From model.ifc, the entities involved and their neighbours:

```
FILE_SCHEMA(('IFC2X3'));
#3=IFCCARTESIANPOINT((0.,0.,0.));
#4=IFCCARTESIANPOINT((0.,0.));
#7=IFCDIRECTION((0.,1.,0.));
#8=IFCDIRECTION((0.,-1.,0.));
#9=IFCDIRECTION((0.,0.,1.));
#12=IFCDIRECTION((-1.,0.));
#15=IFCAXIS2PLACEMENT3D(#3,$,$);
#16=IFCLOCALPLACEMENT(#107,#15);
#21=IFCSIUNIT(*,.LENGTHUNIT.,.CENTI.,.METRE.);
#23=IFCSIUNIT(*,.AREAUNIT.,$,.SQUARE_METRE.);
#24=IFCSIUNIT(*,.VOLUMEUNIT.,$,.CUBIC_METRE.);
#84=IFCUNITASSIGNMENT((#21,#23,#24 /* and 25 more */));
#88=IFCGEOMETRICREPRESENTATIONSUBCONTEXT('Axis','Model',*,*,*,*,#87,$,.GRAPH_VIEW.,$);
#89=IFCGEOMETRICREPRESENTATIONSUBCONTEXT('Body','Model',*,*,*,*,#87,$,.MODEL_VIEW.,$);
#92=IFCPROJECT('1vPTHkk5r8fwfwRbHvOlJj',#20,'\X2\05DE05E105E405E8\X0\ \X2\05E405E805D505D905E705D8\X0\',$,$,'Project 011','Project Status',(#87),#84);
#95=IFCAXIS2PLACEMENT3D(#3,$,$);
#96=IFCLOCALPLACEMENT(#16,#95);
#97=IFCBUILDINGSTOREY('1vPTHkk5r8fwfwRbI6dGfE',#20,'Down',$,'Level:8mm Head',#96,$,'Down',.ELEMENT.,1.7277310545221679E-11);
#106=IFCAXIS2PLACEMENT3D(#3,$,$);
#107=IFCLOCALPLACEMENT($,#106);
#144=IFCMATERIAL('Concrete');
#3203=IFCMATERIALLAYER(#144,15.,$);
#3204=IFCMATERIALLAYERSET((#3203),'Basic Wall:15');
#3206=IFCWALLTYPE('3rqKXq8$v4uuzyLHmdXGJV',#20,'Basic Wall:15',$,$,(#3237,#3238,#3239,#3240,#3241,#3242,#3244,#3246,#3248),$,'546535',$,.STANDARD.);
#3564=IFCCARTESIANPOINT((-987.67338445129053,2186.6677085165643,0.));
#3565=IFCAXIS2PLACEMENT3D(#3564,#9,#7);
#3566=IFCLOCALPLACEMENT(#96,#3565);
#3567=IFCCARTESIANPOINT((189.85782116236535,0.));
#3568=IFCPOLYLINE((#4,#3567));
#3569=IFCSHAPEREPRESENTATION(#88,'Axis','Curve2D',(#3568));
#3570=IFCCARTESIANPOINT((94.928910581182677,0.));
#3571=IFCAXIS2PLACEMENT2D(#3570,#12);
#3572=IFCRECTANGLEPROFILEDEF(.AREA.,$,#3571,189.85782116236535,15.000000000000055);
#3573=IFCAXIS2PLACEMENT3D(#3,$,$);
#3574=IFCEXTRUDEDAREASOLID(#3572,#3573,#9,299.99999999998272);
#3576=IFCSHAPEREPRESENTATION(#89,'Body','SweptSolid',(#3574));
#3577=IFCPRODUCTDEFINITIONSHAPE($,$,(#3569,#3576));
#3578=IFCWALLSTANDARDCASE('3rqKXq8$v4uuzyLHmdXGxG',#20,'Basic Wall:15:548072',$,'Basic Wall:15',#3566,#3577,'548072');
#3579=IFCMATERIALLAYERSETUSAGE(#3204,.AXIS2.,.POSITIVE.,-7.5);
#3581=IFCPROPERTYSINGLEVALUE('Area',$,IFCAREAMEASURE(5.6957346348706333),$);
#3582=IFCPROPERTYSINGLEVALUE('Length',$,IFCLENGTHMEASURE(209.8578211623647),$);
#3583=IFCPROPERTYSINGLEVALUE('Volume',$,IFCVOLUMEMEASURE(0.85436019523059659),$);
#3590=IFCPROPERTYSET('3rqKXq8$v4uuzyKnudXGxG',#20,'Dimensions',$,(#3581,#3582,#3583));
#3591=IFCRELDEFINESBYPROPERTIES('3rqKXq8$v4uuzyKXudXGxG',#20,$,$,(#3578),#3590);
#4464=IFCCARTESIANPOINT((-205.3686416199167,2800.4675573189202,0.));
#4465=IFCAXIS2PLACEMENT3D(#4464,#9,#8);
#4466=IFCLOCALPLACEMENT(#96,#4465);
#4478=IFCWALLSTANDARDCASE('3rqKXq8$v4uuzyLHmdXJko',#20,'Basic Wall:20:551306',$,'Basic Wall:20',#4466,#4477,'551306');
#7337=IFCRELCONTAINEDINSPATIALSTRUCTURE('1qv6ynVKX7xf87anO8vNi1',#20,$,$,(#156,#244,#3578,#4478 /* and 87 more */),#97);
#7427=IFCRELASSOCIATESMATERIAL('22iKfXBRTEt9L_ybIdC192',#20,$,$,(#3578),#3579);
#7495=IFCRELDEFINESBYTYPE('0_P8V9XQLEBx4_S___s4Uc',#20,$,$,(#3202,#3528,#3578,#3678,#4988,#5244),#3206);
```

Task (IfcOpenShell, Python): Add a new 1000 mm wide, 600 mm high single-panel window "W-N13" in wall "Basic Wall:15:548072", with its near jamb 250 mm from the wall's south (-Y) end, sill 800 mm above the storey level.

```python
import numpy as np
import ifcopenshell
import ifcopenshell.api.feature
import ifcopenshell.api.geometry
import ifcopenshell.api.pset
import ifcopenshell.api.root
import ifcopenshell.api.spatial
import ifcopenshell.api.type
import ifcopenshell.geom
import ifcopenshell.util.element
import ifcopenshell.util.placement
import ifcopenshell.util.representation
import ifcopenshell.util.shape
import ifcopenshell.util.unit

model = ifcopenshell.open("model.ifc")
unit_scale = ifcopenshell.util.unit.calculate_unit_scale(model)
area_scale = ifcopenshell.util.unit.calculate_unit_scale(model, "AREAUNIT")
volume_scale = ifcopenshell.util.unit.calculate_unit_scale(model, "VOLUMEUNIT")
settings = ifcopenshell.geom.settings()


def volume(element):
    """Net volume in cubic metres, openings subtracted."""
    shape = ifcopenshell.geom.create_shape(settings, element)
    return ifcopenshell.util.shape.get_volume(shape.geometry)


wall = model.by_id(3578)
storey = ifcopenshell.util.element.get_container(wall, ifc_class="IfcBuildingStorey")
context = ifcopenshell.util.representation.get_context(model, "Model", "Body", "MODEL_VIEW")
before = volume(wall)

width, height, from_end, sill = 1, 0.6, 0.25, 0.8  # metres

# The wall runs along its own X axis, and the end named is its -X end.
wall_shape = ifcopenshell.geom.create_shape(settings, wall)
x, y, z = ifcopenshell.util.shape.get_vertices(wall_shape.geometry).T
start = x.min() + from_end
face, thickness = float(y.min()), float(y.max() - y.min())
wall_matrix = ifcopenshell.util.placement.get_local_placement(wall.ObjectPlacement)
level = ifcopenshell.util.placement.get_local_placement(storey.ObjectPlacement)[2, 3]


def in_wall(x, y):
    """Placement at x, y metres in the wall's axes, at sill height."""
    matrix = wall_matrix.copy()
    matrix[:, 3] = wall_matrix @ np.array([x / unit_scale, y / unit_scale, 0.0, 1.0])
    matrix[2, 3] = level + sill / unit_scale
    return matrix


# Opening: a box that overshoots both wall faces by 50 mm.
opening = ifcopenshell.api.root.create_entity(model, ifc_class="IfcOpeningElement")
box = ifcopenshell.api.geometry.add_wall_representation(
    model, context=context, length=width, height=height, thickness=thickness + 0.1
)
ifcopenshell.api.geometry.assign_representation(model, product=opening, representation=box)
ifcopenshell.api.geometry.edit_object_placement(model, product=opening, matrix=in_wall(start, face - 0.05), is_si=False)
ifcopenshell.api.feature.add_feature(model, feature=opening, element=wall)

window = ifcopenshell.api.root.create_entity(model, ifc_class="IfcWindow", name="W-N13")
window.OverallWidth, window.OverallHeight = width / unit_scale, height / unit_scale
body = ifcopenshell.api.geometry.add_window_representation(
    model,
    context=context,
    overall_width=window.OverallWidth,
    overall_height=window.OverallHeight,
    partition_type="SINGLE_PANEL",
)
ifcopenshell.api.geometry.assign_representation(model, product=window, representation=body)
ifcopenshell.api.spatial.assign_container(model, products=[window], relating_structure=storey)
fills = ifcopenshell.api.feature.add_filling(model, opening=opening, element=window)
fills.OwnerHistory = window.OwnerHistory  # required in IFC2X3

# IFC2X3 keeps the operation on the window style.
style = ifcopenshell.api.root.create_entity(model, ifc_class="IfcWindowStyle", name="W-N13")
style.OperationType, style.ConstructionType = "SINGLE_PANEL", "NOTDEFINED"
style.ParameterTakesPrecedence = style.Sizeable = False
ifcopenshell.api.type.assign_type(model, related_objects=[window], relating_type=style)

# Centre the window in the wall's thickness.
ifcopenshell.api.geometry.edit_object_placement(model, product=window, matrix=in_wall(start, face), is_si=False)
window_shape = ifcopenshell.geom.create_shape(settings, window)
depth = ifcopenshell.util.shape.get_vertices(window_shape.geometry)[:, 1]
offset = face + thickness / 2 - (depth.min() + depth.max()) / 2
ifcopenshell.api.geometry.edit_object_placement(model, product=window, matrix=in_wall(start, offset), is_si=False)

after = volume(wall)

# Update the wall's stored quantities.
pset = model.by_id(ifcopenshell.util.element.get_pset(wall, "Dimensions", should_inherit=False)["id"])
ifcopenshell.api.pset.edit_pset(model, pset=pset, properties={
    "Area": model.create_entity("IfcAreaMeasure", after / thickness / area_scale),
    "Volume": model.create_entity("IfcVolumeMeasure", after / volume_scale),
})

print(f"wall volume {before:.3f} -> {after:.3f} m3")

model.write("model_edited.ifc")
```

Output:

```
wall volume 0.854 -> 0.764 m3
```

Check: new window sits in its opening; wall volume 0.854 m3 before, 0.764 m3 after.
